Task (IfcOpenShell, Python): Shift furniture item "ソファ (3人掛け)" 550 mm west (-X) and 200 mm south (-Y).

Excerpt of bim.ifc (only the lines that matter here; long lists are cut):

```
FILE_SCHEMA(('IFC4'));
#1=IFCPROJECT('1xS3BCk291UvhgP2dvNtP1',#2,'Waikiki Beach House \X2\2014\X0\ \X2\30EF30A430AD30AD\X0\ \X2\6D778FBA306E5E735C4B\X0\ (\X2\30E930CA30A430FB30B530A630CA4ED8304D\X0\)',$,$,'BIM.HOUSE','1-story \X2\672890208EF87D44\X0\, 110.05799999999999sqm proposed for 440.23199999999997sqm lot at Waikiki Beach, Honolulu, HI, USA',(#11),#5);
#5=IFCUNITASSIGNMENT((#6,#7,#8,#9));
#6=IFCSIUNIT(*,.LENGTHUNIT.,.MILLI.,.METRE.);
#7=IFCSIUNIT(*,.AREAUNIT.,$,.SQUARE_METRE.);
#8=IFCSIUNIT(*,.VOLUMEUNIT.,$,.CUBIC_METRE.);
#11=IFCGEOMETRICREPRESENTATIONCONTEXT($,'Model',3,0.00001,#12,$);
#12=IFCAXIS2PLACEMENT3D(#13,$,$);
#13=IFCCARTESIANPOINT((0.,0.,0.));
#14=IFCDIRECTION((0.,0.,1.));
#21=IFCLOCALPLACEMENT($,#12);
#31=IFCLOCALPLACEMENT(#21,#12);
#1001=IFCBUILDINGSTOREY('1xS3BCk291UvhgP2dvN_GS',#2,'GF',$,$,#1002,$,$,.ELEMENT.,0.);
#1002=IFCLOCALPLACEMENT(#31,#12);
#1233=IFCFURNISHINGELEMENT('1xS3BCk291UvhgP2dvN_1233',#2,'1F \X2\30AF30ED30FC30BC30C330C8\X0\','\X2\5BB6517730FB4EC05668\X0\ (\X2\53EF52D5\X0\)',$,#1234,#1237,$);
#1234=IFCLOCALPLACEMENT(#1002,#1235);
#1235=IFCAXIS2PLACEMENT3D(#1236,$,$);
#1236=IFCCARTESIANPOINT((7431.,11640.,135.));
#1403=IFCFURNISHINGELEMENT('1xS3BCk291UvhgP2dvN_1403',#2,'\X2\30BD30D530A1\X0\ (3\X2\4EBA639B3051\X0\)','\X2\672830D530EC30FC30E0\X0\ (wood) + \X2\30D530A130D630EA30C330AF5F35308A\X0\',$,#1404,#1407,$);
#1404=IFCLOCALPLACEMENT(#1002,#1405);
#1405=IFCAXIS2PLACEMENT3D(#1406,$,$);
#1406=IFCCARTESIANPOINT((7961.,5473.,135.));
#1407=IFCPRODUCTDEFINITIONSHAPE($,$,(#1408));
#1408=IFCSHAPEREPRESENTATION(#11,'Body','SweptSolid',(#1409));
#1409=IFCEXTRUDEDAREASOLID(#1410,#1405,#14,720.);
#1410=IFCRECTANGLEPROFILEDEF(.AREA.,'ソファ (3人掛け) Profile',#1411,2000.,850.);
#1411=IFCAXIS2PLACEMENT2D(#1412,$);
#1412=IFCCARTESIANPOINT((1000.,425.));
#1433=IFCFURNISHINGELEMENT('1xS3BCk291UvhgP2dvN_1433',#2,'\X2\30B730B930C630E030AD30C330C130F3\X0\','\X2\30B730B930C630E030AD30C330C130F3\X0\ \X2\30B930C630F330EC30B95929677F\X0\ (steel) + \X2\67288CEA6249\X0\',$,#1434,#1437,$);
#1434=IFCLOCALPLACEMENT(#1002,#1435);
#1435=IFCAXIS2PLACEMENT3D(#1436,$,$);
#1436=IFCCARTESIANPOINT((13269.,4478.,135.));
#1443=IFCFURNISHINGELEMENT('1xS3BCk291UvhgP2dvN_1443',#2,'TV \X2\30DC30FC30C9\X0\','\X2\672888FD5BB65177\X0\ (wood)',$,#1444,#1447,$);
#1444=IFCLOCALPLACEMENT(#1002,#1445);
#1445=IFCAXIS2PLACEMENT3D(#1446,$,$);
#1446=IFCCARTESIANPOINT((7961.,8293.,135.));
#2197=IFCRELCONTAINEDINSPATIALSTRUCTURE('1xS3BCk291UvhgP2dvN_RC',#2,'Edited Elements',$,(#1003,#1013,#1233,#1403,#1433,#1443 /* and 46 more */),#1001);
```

```python
import ifcopenshell
import ifcopenshell.api.geometry
import ifcopenshell.util.placement
import ifcopenshell.util.unit

model = ifcopenshell.open("bim.ifc")
unit_scale = ifcopenshell.util.unit.calculate_unit_scale(model)

item = model.by_id(1403)
matrix = ifcopenshell.util.placement.get_local_placement(item.ObjectPlacement)
matrix[0, 3] -= 0.55 / unit_scale
matrix[1, 3] -= 0.2 / unit_scale
ifcopenshell.api.geometry.edit_object_placement(model, product=item, matrix=matrix, is_si=False)

print(ifcopenshell.util.placement.get_local_placement(item.ObjectPlacement).round(3) + 0.0)

model.write("bim_updated.ifc")
```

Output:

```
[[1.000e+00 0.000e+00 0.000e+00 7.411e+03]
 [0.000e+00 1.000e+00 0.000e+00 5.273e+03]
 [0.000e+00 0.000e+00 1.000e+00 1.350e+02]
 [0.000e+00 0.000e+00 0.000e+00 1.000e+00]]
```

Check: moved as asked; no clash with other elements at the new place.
